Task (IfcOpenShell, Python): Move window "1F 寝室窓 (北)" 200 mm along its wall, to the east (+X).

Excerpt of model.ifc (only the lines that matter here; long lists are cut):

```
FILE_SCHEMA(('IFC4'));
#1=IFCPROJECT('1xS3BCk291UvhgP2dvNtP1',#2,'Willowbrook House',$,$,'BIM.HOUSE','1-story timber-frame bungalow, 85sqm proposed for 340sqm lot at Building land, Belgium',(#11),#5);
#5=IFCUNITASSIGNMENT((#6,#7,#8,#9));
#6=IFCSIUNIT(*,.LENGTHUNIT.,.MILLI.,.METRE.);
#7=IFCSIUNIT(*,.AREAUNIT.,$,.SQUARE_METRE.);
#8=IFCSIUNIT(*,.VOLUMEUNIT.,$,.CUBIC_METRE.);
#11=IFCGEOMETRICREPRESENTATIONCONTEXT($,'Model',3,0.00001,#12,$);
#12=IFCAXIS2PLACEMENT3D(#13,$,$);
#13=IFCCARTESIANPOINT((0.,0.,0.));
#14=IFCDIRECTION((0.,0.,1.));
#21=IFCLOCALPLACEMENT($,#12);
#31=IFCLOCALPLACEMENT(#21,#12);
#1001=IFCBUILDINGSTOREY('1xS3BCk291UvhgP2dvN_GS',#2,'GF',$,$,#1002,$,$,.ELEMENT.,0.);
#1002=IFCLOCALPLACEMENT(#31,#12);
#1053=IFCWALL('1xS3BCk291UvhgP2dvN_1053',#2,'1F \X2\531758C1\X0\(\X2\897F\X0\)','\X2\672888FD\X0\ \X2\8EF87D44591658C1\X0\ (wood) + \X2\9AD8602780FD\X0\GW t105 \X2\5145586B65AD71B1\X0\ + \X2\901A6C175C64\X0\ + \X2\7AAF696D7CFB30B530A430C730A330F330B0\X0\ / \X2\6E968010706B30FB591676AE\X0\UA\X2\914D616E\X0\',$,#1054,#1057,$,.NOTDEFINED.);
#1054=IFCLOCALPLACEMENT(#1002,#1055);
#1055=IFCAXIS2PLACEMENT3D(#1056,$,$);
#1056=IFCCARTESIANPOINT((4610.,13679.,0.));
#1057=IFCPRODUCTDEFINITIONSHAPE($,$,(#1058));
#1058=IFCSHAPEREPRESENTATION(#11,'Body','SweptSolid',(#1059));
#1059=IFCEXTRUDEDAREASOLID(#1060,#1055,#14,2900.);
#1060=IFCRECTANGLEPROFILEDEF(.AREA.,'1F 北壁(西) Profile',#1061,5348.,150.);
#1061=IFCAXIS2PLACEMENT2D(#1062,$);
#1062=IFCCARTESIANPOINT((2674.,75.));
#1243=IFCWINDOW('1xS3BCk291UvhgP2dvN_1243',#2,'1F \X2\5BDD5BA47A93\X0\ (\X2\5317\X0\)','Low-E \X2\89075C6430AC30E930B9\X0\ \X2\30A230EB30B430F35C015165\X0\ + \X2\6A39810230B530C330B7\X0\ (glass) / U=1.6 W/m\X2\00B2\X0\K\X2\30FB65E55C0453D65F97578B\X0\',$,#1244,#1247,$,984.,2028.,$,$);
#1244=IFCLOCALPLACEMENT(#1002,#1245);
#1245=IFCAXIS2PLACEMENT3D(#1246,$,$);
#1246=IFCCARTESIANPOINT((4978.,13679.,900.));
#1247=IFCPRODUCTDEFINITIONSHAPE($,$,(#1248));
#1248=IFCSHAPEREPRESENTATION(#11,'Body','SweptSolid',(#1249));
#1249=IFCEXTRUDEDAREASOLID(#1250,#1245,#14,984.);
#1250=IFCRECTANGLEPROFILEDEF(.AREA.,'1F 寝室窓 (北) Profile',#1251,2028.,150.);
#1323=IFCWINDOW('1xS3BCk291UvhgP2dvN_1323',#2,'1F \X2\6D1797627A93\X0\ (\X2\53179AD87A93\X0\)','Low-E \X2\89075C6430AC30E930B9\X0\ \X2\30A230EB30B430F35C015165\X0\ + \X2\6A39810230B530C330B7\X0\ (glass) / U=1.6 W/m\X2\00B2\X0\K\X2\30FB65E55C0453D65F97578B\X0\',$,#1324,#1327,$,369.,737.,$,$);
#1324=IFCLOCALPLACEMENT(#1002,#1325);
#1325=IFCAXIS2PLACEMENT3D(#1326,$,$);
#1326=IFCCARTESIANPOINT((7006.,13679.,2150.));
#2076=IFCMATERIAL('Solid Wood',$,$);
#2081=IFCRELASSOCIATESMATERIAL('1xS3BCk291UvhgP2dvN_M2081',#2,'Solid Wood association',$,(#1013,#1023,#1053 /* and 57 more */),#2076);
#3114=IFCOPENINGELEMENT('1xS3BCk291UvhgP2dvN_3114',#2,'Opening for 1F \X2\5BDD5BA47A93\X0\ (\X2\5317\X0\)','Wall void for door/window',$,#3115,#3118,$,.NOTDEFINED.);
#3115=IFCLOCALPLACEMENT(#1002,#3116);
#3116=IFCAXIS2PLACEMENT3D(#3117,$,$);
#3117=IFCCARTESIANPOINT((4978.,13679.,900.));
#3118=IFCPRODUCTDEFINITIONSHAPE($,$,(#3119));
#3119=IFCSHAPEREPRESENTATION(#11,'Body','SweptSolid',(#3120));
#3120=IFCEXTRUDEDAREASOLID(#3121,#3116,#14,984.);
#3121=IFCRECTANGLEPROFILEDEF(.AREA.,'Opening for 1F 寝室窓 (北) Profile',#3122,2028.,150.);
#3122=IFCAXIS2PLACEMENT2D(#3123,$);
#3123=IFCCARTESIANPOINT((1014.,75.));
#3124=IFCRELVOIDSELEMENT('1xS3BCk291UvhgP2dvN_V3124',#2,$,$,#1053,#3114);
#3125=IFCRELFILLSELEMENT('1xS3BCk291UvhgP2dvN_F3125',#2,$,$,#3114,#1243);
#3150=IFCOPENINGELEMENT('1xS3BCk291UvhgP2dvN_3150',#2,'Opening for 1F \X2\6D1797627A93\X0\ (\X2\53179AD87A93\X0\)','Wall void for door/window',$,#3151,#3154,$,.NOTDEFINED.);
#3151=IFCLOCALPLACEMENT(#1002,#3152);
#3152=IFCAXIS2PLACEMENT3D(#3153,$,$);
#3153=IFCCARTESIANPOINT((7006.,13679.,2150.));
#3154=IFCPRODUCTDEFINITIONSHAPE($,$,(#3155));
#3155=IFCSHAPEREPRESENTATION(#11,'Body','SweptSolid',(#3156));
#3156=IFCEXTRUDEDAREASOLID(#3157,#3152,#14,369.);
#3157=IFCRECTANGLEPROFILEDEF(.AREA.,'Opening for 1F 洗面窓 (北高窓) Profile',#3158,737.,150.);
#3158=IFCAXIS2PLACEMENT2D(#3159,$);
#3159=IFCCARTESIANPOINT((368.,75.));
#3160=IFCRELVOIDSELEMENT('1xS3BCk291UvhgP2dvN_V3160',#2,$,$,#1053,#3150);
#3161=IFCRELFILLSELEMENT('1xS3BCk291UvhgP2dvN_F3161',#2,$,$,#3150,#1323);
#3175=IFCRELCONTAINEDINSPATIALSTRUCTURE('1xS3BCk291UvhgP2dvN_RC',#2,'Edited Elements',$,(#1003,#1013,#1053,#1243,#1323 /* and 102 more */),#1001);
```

```python
import ifcopenshell
import ifcopenshell.api.geometry
import ifcopenshell.util.placement
import ifcopenshell.util.unit

model = ifcopenshell.open("model.ifc")
unit_scale = ifcopenshell.util.unit.calculate_unit_scale(model)

window = model.by_id(1243)
opening = window.FillsVoids[0].RelatingOpeningElement
wall = opening.VoidsElements[0].RelatingBuildingElement

wall_matrix = ifcopenshell.util.placement.get_local_placement(wall.ObjectPlacement)
shift = wall_matrix[:3, 0] * 0.2 / unit_scale
before = ifcopenshell.util.placement.get_local_placement(window.ObjectPlacement)[:3, 3].copy()

# The window is not placed relative to its opening, so move both.
for product in (opening, window):
    matrix = ifcopenshell.util.placement.get_local_placement(product.ObjectPlacement)
    matrix[:3, 3] += shift
    ifcopenshell.api.geometry.edit_object_placement(model, product=product, matrix=matrix, is_si=False)

after = ifcopenshell.util.placement.get_local_placement(window.ObjectPlacement)[:3, 3]
print("window moved by", (after - before).round(3) + 0.0)

model.write("model_v2.ifc")
```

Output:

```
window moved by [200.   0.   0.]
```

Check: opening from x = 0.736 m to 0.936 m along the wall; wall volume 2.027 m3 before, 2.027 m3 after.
